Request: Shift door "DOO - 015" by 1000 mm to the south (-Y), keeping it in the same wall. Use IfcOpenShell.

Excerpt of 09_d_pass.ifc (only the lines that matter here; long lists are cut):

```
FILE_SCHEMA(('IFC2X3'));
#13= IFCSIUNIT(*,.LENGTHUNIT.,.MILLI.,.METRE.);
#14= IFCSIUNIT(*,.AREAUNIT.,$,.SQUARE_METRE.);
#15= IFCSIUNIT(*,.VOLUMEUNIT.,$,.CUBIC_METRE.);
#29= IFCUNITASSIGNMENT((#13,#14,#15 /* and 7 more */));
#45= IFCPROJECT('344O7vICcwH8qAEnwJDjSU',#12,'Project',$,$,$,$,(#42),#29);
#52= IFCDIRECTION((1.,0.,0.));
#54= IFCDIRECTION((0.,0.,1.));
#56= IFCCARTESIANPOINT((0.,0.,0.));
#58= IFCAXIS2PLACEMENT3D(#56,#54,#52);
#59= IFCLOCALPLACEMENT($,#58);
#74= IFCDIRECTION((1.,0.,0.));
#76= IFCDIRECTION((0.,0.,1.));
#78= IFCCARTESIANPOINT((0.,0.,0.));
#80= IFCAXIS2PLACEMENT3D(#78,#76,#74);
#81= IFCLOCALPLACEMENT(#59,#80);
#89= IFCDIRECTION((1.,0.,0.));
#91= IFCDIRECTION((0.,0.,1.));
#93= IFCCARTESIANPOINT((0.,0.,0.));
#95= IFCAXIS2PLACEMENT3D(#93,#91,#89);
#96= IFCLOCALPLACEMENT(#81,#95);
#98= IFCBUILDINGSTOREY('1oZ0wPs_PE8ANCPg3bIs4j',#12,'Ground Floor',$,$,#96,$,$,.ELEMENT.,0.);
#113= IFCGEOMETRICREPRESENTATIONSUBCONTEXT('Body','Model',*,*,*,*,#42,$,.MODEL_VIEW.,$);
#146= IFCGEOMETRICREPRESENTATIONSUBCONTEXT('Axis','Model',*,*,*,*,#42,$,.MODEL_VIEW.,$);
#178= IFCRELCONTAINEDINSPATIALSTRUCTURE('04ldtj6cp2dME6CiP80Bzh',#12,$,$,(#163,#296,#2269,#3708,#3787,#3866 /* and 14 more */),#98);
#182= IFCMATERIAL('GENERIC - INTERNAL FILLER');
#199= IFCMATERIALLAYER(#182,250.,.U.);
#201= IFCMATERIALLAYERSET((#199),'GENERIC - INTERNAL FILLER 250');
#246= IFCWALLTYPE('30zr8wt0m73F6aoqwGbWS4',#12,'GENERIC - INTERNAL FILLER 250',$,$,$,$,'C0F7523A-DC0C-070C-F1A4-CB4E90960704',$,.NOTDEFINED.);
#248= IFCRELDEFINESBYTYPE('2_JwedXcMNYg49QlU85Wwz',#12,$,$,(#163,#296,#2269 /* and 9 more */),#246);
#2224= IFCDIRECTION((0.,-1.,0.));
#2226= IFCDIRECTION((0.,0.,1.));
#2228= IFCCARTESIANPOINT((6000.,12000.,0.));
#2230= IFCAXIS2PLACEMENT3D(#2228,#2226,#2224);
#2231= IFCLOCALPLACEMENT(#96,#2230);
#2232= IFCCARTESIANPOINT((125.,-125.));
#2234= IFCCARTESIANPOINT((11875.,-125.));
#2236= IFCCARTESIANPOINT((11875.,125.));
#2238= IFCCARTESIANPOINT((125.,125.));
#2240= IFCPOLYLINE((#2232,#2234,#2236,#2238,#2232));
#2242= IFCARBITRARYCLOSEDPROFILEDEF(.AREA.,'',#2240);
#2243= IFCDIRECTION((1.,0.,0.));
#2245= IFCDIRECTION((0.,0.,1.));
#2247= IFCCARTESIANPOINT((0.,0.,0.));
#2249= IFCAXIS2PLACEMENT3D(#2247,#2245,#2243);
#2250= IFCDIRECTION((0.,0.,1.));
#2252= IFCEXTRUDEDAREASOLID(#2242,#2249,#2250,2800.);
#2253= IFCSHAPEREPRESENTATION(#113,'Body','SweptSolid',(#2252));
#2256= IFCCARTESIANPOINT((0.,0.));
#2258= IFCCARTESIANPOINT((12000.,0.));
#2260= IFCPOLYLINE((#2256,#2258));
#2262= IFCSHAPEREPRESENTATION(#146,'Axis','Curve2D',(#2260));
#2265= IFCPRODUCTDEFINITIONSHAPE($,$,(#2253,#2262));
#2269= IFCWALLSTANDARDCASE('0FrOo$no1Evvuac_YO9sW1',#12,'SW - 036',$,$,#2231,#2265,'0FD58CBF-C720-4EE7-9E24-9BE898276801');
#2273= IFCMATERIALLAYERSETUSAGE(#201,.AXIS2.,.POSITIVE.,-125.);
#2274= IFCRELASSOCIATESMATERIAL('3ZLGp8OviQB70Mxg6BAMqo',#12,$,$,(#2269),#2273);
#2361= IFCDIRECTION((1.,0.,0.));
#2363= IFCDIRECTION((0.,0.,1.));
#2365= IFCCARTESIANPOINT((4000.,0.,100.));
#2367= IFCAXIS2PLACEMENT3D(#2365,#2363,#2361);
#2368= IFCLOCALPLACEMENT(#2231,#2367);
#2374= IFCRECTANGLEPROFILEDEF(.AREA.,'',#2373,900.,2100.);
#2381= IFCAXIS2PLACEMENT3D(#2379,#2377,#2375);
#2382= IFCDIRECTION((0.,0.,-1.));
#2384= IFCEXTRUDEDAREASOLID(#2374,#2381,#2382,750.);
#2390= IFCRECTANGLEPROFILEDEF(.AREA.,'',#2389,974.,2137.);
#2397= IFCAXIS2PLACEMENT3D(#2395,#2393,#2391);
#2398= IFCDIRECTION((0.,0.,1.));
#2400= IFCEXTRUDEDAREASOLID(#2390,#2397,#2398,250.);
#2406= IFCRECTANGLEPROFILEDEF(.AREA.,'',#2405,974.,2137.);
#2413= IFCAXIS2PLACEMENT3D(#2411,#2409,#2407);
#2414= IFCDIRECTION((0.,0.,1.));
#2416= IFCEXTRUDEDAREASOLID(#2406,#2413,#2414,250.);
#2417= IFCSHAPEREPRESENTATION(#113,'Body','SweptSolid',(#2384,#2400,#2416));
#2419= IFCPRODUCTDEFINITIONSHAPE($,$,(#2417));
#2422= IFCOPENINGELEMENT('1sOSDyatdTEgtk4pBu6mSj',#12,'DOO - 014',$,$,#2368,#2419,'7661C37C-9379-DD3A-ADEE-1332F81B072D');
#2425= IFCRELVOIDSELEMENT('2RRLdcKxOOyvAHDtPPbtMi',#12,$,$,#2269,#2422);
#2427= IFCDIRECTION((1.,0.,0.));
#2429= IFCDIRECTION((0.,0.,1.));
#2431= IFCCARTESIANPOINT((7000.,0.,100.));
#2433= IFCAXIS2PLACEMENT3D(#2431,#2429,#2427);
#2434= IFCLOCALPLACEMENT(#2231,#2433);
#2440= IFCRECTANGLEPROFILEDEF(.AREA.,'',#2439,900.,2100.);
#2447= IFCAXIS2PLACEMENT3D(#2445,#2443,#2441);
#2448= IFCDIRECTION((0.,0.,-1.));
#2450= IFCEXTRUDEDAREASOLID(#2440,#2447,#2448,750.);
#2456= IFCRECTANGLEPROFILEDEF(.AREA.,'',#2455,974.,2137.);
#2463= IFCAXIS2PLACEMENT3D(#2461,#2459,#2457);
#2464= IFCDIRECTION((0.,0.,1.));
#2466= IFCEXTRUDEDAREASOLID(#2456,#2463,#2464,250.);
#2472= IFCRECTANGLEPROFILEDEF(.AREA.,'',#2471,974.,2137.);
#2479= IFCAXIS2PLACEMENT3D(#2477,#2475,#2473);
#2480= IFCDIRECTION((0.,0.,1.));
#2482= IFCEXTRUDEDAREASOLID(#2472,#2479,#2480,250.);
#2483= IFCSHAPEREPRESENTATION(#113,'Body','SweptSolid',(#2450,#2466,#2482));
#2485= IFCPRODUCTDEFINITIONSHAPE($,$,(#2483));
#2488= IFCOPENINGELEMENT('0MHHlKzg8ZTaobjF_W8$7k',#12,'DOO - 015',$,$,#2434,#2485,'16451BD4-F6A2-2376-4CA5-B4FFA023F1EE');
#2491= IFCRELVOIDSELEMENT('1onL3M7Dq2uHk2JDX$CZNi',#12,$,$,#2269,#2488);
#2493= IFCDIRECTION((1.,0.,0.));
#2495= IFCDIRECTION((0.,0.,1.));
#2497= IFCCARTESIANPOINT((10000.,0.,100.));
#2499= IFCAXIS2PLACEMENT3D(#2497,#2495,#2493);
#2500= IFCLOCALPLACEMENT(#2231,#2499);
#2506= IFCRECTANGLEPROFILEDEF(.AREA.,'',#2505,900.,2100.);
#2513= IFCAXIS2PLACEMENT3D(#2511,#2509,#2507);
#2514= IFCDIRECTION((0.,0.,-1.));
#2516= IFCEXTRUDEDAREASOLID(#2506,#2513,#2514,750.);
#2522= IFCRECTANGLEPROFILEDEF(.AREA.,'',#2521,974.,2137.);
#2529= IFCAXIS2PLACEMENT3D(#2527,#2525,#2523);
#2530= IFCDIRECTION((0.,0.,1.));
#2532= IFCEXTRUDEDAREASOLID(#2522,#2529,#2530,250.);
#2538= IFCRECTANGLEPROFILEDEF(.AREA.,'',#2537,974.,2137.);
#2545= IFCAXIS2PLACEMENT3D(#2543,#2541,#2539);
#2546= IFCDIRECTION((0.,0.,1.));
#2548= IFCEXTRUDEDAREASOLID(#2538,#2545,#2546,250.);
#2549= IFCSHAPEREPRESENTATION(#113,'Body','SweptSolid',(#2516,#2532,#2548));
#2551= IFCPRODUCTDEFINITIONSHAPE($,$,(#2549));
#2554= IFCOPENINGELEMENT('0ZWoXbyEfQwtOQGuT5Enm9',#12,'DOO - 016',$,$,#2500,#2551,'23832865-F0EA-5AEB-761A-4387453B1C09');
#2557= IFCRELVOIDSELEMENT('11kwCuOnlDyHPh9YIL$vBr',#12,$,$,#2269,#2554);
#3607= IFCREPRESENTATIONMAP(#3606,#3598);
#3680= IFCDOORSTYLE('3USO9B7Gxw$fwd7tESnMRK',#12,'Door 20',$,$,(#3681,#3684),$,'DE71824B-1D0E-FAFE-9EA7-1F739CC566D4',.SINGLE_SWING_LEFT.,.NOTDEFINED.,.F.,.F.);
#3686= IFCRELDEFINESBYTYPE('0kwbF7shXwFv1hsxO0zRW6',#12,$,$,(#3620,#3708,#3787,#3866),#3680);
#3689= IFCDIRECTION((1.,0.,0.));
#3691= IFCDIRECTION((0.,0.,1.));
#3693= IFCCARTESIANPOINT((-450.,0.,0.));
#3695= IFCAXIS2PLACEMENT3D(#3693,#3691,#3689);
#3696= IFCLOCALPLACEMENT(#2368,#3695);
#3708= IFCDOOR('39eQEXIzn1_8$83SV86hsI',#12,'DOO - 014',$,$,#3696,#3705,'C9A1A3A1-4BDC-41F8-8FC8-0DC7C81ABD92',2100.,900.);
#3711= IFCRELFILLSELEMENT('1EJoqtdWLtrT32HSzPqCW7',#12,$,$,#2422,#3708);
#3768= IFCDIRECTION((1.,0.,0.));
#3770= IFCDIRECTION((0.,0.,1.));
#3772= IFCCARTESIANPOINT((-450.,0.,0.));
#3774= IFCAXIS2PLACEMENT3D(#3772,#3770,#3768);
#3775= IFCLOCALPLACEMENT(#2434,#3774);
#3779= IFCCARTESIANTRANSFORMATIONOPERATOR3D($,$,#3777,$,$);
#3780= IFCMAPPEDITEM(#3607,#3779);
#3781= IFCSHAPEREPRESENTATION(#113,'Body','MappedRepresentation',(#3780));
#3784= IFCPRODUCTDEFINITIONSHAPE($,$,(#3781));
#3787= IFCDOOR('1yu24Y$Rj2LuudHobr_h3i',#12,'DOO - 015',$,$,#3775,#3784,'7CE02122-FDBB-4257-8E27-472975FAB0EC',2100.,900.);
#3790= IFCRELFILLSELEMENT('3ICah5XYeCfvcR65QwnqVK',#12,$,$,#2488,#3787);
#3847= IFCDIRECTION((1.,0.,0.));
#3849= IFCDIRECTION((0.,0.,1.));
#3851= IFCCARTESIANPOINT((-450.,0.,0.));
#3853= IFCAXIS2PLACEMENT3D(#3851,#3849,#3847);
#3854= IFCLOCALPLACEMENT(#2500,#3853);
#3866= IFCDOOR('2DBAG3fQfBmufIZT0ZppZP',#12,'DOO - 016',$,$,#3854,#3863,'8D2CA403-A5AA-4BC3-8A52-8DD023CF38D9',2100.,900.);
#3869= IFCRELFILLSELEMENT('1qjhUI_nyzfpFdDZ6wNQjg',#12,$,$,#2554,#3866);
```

```python
import ifcopenshell
import ifcopenshell.api.geometry
import ifcopenshell.util.placement
import ifcopenshell.util.unit

model = ifcopenshell.open("09_d_pass.ifc")
unit_scale = ifcopenshell.util.unit.calculate_unit_scale(model)

door = model.by_id(3787)
opening = door.FillsVoids[0].RelatingOpeningElement
wall = opening.VoidsElements[0].RelatingBuildingElement

wall_matrix = ifcopenshell.util.placement.get_local_placement(wall.ObjectPlacement)
shift = wall_matrix[:3, 0] * 1 / unit_scale
before = ifcopenshell.util.placement.get_local_placement(door.ObjectPlacement)[:3, 3].copy()

# The door is placed relative to its opening, so it follows when the opening moves.
matrix = ifcopenshell.util.placement.get_local_placement(opening.ObjectPlacement)
matrix[:3, 3] += shift
ifcopenshell.api.geometry.edit_object_placement(
    model, product=opening, matrix=matrix, is_si=False, should_transform_children=True
)

after = ifcopenshell.util.placement.get_local_placement(door.ObjectPlacement)[:3, 3]
print("door moved by", (after - before).round(3) + 0.0)

model.write("09_d_pass_edited.ifc")
```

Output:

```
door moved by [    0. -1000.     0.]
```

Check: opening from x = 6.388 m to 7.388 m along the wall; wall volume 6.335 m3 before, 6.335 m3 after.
